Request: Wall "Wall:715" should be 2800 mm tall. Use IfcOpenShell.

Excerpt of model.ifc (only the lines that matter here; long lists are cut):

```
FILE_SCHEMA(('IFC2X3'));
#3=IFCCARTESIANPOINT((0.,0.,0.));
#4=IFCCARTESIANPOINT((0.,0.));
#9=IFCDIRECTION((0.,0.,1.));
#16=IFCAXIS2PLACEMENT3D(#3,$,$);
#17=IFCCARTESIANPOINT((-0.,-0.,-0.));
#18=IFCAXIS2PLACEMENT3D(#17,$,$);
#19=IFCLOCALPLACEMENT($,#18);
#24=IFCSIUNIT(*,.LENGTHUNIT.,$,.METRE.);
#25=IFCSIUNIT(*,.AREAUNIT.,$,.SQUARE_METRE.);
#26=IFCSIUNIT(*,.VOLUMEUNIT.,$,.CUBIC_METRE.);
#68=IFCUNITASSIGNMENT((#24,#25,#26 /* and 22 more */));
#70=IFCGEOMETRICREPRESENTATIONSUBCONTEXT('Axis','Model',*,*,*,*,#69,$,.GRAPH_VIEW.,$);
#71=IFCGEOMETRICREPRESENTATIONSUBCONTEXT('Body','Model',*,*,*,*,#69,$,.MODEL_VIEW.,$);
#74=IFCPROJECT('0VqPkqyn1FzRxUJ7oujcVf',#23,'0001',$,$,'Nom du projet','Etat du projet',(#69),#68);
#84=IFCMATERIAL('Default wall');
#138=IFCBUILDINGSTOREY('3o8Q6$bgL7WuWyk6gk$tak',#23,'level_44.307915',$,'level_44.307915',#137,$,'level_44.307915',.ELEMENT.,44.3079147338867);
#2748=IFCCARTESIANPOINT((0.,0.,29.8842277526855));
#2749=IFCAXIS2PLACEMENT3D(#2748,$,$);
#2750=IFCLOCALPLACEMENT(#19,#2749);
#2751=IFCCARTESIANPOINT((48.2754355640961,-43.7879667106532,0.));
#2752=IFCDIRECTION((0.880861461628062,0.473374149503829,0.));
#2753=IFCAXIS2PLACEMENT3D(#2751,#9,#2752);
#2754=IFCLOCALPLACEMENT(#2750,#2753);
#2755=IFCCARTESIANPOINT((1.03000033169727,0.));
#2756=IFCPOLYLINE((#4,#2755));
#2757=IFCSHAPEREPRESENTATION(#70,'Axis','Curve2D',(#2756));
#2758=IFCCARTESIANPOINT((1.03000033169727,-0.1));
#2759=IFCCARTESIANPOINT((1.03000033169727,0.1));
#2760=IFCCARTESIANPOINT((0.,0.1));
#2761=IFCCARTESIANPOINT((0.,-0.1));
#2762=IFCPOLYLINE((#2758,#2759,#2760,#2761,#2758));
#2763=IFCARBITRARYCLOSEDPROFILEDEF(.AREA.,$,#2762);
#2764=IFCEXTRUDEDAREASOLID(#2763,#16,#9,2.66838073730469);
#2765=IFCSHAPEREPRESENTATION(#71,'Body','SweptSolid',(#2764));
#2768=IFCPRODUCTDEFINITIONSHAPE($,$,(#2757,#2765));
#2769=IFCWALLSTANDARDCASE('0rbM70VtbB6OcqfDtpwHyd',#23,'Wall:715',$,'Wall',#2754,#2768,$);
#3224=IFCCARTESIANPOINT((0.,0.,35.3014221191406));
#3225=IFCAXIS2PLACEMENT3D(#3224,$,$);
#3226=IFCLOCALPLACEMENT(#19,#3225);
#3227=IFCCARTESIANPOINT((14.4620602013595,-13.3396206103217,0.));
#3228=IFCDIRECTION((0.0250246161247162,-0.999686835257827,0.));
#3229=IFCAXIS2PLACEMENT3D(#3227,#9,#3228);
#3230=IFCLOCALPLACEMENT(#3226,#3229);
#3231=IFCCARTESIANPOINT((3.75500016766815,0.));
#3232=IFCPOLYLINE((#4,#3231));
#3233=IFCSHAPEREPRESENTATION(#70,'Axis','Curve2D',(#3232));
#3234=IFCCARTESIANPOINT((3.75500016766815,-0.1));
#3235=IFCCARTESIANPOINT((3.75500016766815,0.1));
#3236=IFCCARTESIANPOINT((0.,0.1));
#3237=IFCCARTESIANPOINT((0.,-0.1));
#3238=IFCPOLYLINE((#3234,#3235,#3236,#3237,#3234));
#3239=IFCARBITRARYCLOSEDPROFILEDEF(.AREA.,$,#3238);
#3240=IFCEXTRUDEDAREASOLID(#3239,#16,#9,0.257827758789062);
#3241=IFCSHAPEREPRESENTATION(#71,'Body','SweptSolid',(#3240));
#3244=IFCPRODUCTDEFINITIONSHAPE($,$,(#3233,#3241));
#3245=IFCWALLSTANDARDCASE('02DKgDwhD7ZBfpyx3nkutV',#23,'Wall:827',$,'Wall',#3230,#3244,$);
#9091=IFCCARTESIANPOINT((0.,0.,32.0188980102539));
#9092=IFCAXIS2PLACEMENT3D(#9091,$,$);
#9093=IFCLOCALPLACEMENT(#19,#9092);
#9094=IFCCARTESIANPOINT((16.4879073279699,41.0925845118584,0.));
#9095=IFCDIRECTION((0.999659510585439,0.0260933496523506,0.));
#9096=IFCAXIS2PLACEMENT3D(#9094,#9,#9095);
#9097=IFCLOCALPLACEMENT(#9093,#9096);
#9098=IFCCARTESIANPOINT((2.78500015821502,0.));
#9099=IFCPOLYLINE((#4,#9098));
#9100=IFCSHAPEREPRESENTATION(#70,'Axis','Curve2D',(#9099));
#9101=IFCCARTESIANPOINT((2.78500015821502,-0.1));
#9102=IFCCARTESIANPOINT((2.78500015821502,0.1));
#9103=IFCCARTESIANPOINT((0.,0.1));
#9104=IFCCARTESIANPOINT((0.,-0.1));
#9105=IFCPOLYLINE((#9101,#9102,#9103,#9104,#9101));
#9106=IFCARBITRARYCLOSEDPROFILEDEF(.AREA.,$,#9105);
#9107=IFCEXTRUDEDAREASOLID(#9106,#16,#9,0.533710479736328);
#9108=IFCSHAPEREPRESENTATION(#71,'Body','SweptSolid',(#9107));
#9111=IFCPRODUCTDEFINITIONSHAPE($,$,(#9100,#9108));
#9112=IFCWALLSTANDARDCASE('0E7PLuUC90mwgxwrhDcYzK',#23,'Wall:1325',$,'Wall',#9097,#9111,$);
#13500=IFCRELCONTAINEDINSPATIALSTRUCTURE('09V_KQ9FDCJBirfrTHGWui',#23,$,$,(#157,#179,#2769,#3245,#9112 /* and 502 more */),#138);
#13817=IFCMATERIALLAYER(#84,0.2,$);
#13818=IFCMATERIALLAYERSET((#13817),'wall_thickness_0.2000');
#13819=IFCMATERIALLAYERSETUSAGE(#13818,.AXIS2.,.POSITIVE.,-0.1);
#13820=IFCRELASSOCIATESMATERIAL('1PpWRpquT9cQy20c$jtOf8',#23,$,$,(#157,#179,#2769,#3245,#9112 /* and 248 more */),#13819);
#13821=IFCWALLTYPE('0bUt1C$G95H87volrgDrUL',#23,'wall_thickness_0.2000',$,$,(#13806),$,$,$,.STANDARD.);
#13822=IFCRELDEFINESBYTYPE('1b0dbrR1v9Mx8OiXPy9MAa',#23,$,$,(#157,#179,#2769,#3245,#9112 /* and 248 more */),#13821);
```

```python
import ifcopenshell
import ifcopenshell.geom
import ifcopenshell.util.representation
import ifcopenshell.util.shape

model = ifcopenshell.open("model.ifc")
settings = ifcopenshell.geom.settings()


def volume(element):
    """Net volume in cubic metres, openings subtracted."""
    shape = ifcopenshell.geom.create_shape(settings, element)
    return ifcopenshell.util.shape.get_volume(shape.geometry)


wall = model.by_guid("0rbM70VtbB6OcqfDtpwHyd")
before = volume(wall)

body = ifcopenshell.util.representation.get_representation(wall, "Model", "Body")
solid = body.Items[0]
old_height = solid.Depth
solid.Depth = 2.8
after = volume(wall)

print(f"height {old_height:g} -> {solid.Depth:g}, volume {before:.3f} -> {after:.3f} m3")

model.write("model_updated.ifc")
```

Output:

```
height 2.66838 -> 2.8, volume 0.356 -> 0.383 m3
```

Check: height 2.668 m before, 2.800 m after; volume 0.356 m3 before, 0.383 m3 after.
